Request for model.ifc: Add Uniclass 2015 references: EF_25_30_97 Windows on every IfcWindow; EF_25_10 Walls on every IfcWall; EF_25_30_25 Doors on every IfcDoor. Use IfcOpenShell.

First a look at what the model holds.

```python
import ifcopenshell

model = ifcopenshell.open("model.ifc")
print(model.schema)
print("classifications:", [c.Name for c in model.by_type("IfcClassification")])
for ifc_class in ("IfcDoor", "IfcRoof", "IfcStair", "IfcWall", "IfcWindow"):
    print(ifc_class, len(model.by_type(ifc_class)))
```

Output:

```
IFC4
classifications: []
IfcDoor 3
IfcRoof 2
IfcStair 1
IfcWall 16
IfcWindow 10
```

```python
import ifcopenshell
import ifcopenshell.api.classification

model = ifcopenshell.open("model.ifc")

system = ifcopenshell.api.classification.add_classification(model, classification="Uniclass 2015")

codes = {
    "IfcWindow": ("EF_25_30_97", "Windows"),
    "IfcWall": ("EF_25_10", "Walls"),
    "IfcDoor": ("EF_25_30_25", "Doors"),
}
for ifc_class, (code, name) in codes.items():
    products = model.by_type(ifc_class)
    ifcopenshell.api.classification.add_reference(
        model, products=products, classification=system, identification=code, name=name
    )
    print(code, len(products))

model.write("model_v2.ifc")
```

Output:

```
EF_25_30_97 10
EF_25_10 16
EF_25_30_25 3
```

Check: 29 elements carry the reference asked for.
